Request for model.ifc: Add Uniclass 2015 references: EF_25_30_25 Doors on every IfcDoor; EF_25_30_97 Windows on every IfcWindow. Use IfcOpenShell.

First a look at what the model holds.

```python
import ifcopenshell

model = ifcopenshell.open("model.ifc")
print(model.schema)
print("classifications:", [c.Name for c in model.by_type("IfcClassification")])
for ifc_class in ("IfcDoor", "IfcRoof", "IfcStair", "IfcWall", "IfcWindow"):
    print(ifc_class, len(model.by_type(ifc_class)))
```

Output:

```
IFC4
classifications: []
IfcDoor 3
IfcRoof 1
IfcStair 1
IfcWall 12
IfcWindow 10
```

```python
import ifcopenshell
import ifcopenshell.api.classification

model = ifcopenshell.open("model.ifc")

system = ifcopenshell.api.classification.add_classification(model, classification="Uniclass 2015")

codes = {
    "IfcDoor": ("EF_25_30_25", "Doors"),
    "IfcWindow": ("EF_25_30_97", "Windows"),
}
for ifc_class, (code, name) in codes.items():
    products = model.by_type(ifc_class)
    ifcopenshell.api.classification.add_reference(
        model, products=products, classification=system, identification=code, name=name
    )
    print(code, len(products))

model.write("model_rev.ifc")
```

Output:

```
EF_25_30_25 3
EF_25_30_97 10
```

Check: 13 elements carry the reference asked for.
